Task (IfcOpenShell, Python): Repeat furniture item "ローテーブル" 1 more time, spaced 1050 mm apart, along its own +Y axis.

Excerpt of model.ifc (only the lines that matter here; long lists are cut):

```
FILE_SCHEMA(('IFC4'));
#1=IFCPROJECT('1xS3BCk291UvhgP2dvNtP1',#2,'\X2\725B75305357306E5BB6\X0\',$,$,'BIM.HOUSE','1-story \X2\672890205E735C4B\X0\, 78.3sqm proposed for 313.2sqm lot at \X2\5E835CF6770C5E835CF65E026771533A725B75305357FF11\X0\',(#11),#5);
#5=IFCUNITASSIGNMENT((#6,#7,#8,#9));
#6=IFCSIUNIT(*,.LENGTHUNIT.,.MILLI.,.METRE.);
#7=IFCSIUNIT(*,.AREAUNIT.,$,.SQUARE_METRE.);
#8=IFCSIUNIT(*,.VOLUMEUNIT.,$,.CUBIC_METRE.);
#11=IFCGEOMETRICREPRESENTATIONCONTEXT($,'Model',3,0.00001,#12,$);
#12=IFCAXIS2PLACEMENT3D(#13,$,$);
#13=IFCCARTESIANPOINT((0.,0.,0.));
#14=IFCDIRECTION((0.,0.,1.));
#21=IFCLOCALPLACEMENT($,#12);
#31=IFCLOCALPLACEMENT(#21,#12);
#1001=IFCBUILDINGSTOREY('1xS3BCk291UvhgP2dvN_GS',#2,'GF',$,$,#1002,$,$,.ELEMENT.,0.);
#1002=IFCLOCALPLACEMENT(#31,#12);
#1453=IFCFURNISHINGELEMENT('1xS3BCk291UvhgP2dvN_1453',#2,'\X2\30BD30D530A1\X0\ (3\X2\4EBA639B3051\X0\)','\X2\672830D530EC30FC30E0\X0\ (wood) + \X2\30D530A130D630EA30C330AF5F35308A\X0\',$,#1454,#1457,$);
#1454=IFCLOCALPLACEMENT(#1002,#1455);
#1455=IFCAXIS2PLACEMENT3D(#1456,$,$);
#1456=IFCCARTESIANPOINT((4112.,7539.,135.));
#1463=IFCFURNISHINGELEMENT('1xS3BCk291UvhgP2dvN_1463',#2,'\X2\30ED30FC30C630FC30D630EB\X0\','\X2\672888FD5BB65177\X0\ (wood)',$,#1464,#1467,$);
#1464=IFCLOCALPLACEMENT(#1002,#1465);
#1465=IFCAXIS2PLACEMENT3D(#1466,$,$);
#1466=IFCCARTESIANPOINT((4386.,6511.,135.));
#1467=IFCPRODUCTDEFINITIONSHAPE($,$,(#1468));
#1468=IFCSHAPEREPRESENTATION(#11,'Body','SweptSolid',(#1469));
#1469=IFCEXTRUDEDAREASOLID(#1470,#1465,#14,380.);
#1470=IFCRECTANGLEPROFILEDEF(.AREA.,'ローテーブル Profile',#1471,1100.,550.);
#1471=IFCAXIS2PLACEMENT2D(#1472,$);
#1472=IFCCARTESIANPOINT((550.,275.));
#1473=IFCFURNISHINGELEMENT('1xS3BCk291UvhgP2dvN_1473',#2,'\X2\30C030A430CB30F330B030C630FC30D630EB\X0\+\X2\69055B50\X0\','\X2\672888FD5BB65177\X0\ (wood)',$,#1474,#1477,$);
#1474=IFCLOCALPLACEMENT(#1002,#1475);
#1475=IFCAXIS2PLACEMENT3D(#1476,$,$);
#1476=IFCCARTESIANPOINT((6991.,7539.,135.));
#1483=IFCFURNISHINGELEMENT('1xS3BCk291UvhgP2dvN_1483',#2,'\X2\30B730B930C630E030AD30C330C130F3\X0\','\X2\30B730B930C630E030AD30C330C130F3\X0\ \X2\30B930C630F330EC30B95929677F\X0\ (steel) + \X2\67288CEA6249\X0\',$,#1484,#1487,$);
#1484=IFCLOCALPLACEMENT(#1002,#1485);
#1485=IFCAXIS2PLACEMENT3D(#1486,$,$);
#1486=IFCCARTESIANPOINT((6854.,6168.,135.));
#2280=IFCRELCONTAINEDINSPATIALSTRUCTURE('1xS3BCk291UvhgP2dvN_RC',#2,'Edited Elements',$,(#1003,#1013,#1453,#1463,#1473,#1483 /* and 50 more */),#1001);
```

```python
import ifcopenshell
import ifcopenshell.api.geometry
import ifcopenshell.api.root
import ifcopenshell.util.element
import ifcopenshell.util.placement
import ifcopenshell.util.unit

model = ifcopenshell.open("model.ifc")
unit_scale = ifcopenshell.util.unit.calculate_unit_scale(model)


def reuse_history(source, copy):
    """copy_class also copies each property set's owner history, people and application; keep the originals."""
    for rel in copy.IsDefinedBy:
        if rel.is_a("IfcRelDefinesByProperties") and (history := rel.RelatingPropertyDefinition.OwnerHistory):
            rel.RelatingPropertyDefinition.OwnerHistory = source.OwnerHistory
            ifcopenshell.util.element.remove_deep2(model, history)


source = model.by_guid("1xS3BCk291UvhgP2dvN_1463")
base = ifcopenshell.util.placement.get_local_placement(source.ObjectPlacement)
step = base[:3, 1] * 1.05 / unit_scale

for i in range(1, 2):
    copy = ifcopenshell.api.root.copy_class(model, product=source)
    copy.Representation = ifcopenshell.util.element.copy_deep(
        model, source.Representation, exclude=["IfcGeometricRepresentationContext", "IfcRepresentationMap"]
    )
    reuse_history(source, copy)
    matrix = base.copy()
    matrix[:3, 3] += i * step
    print("added at", matrix[:3, 3].round(3) + 0.0)
    ifcopenshell.api.geometry.edit_object_placement(model, product=copy, matrix=matrix, is_si=False)

model.write("model-out.ifc")
```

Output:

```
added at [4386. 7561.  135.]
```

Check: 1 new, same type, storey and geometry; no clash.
